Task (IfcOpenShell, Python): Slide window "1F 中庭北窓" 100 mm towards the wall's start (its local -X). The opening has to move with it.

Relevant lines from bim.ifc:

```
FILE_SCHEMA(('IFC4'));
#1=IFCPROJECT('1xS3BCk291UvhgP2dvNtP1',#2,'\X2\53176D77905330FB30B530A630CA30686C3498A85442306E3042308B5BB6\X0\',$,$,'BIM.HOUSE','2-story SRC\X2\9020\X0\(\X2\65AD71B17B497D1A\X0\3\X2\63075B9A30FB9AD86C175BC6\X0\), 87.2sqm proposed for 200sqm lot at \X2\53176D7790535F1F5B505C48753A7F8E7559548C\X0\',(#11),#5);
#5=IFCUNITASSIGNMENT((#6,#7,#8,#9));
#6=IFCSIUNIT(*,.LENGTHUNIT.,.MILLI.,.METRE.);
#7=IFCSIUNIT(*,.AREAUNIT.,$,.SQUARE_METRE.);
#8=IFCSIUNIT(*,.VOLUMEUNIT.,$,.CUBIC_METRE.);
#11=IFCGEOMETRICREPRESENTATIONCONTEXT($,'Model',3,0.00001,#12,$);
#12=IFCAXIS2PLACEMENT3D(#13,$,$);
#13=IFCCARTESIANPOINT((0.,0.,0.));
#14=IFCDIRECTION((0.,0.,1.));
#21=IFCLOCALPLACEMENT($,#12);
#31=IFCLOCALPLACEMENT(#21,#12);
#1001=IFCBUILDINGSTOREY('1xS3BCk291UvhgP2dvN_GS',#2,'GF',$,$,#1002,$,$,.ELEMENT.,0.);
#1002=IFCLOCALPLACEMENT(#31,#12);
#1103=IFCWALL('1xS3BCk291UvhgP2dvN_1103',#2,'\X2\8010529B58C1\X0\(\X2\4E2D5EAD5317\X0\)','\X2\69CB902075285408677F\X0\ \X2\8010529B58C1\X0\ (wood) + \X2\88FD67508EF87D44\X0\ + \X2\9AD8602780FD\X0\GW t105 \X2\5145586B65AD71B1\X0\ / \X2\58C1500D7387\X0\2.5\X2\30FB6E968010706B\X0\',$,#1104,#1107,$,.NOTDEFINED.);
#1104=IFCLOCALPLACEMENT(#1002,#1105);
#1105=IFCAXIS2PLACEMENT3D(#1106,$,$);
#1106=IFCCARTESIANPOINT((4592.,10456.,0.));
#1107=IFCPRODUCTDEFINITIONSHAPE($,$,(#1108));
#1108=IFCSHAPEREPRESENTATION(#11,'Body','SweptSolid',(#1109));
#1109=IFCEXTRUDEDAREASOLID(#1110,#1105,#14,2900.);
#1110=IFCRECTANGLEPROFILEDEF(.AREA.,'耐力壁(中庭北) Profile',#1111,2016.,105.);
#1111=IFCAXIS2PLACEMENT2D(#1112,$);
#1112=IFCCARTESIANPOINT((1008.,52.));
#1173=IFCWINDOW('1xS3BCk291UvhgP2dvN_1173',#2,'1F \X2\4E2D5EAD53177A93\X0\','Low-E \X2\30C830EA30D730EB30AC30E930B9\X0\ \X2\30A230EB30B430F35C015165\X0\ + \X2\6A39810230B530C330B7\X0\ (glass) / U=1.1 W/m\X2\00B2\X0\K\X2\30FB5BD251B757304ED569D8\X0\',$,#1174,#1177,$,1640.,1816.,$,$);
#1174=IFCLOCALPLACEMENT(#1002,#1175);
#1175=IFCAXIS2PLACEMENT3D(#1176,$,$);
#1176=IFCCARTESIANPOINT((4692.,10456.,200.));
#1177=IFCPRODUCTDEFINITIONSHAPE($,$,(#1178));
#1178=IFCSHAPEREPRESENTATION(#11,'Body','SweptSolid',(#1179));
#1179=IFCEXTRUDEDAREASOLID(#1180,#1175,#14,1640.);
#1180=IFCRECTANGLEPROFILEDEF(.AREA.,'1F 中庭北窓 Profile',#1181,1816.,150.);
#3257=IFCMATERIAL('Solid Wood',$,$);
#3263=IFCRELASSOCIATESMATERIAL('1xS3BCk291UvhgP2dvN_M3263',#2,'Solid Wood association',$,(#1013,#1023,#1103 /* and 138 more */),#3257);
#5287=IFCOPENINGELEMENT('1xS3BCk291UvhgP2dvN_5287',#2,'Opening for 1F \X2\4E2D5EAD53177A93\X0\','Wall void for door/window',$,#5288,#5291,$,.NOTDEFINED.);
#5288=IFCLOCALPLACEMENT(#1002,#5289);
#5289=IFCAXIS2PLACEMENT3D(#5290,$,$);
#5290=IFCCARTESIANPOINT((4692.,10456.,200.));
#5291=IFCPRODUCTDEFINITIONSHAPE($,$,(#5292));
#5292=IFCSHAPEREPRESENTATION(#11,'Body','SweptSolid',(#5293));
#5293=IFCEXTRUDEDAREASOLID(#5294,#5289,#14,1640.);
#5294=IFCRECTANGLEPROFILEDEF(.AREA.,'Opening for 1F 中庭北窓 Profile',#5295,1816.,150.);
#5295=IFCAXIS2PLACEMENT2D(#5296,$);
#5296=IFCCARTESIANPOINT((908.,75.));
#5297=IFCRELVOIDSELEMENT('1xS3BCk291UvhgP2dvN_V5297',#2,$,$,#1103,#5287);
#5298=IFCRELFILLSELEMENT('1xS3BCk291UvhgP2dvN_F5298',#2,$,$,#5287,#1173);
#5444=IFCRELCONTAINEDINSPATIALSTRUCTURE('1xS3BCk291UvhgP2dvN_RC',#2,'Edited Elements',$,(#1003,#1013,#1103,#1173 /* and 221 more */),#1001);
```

```python
import ifcopenshell
import ifcopenshell.api.geometry
import ifcopenshell.util.placement
import ifcopenshell.util.unit

model = ifcopenshell.open("bim.ifc")
unit_scale = ifcopenshell.util.unit.calculate_unit_scale(model)

window = model.by_id(1173)
opening = window.FillsVoids[0].RelatingOpeningElement
wall = opening.VoidsElements[0].RelatingBuildingElement

wall_matrix = ifcopenshell.util.placement.get_local_placement(wall.ObjectPlacement)
shift = wall_matrix[:3, 0] * -0.1 / unit_scale
before = ifcopenshell.util.placement.get_local_placement(window.ObjectPlacement)[:3, 3].copy()

# The window is not placed relative to its opening, so move both.
for product in (opening, window):
    matrix = ifcopenshell.util.placement.get_local_placement(product.ObjectPlacement)
    matrix[:3, 3] += shift
    ifcopenshell.api.geometry.edit_object_placement(model, product=product, matrix=matrix, is_si=False)

after = ifcopenshell.util.placement.get_local_placement(window.ObjectPlacement)[:3, 3]
print("window moved by", (after - before).round(3) + 0.0)

model.write("bim-out.ifc")
```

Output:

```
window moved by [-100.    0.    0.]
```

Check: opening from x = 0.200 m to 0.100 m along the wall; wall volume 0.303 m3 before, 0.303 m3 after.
